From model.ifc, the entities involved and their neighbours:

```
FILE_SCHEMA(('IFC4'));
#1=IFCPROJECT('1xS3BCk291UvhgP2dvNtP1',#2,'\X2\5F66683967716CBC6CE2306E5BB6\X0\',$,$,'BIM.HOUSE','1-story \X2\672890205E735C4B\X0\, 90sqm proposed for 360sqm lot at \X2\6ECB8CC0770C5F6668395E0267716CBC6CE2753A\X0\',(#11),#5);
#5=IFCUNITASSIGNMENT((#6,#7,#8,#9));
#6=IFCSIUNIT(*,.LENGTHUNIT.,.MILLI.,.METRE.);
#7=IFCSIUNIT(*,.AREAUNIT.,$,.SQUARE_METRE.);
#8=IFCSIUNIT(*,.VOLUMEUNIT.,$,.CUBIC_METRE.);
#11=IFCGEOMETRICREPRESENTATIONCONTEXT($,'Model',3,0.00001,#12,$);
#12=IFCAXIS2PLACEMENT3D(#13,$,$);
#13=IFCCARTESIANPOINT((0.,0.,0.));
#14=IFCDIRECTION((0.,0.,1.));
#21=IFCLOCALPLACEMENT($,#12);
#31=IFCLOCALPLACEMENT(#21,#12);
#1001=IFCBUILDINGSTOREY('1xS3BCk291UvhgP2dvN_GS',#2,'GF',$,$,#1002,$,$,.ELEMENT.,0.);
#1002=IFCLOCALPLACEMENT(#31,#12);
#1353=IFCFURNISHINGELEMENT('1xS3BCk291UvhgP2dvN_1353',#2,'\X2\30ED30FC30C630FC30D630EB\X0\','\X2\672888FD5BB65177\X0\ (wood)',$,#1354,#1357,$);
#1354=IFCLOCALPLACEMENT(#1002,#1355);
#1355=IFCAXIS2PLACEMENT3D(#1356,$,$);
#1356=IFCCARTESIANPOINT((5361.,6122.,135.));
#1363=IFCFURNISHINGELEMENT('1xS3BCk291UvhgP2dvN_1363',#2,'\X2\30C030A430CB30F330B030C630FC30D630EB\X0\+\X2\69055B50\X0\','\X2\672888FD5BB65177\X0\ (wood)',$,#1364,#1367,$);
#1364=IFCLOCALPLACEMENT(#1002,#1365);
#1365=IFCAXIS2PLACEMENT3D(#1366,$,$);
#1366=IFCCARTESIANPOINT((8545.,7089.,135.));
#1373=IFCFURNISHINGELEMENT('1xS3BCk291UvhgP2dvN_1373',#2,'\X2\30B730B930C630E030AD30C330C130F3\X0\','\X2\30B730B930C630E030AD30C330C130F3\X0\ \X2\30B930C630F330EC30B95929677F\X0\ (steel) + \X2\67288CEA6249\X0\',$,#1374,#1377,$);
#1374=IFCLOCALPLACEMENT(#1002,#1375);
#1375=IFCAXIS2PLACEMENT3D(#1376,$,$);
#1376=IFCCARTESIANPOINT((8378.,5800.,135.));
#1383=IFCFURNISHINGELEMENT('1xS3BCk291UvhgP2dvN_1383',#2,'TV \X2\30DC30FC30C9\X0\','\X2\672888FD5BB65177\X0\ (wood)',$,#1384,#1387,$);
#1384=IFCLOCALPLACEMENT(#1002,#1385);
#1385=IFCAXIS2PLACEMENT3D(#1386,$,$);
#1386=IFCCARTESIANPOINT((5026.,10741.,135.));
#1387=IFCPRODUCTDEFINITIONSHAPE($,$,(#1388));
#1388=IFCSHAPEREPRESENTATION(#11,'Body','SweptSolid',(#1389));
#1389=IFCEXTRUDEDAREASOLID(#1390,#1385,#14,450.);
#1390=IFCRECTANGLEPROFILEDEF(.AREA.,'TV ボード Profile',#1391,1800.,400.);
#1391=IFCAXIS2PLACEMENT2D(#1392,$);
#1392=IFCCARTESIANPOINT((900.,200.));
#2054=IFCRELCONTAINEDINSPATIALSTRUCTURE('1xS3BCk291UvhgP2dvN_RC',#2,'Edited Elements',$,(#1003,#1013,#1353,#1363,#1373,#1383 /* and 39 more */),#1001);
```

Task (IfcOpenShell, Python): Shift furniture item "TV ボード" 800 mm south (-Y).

```python
import ifcopenshell
import ifcopenshell.api.geometry
import ifcopenshell.util.placement
import ifcopenshell.util.unit

model = ifcopenshell.open("model.ifc")
unit_scale = ifcopenshell.util.unit.calculate_unit_scale(model)

item = model.by_guid("1xS3BCk291UvhgP2dvN_1383")
matrix = ifcopenshell.util.placement.get_local_placement(item.ObjectPlacement)
matrix[1, 3] -= 0.8 / unit_scale
ifcopenshell.api.geometry.edit_object_placement(model, product=item, matrix=matrix, is_si=False)

print(ifcopenshell.util.placement.get_local_placement(item.ObjectPlacement).round(3) + 0.0)

model.write("model-out.ifc")
```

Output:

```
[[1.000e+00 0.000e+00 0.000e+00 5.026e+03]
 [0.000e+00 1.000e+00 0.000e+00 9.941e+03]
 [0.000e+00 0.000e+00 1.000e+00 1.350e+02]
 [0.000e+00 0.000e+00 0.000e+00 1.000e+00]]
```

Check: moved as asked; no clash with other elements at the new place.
